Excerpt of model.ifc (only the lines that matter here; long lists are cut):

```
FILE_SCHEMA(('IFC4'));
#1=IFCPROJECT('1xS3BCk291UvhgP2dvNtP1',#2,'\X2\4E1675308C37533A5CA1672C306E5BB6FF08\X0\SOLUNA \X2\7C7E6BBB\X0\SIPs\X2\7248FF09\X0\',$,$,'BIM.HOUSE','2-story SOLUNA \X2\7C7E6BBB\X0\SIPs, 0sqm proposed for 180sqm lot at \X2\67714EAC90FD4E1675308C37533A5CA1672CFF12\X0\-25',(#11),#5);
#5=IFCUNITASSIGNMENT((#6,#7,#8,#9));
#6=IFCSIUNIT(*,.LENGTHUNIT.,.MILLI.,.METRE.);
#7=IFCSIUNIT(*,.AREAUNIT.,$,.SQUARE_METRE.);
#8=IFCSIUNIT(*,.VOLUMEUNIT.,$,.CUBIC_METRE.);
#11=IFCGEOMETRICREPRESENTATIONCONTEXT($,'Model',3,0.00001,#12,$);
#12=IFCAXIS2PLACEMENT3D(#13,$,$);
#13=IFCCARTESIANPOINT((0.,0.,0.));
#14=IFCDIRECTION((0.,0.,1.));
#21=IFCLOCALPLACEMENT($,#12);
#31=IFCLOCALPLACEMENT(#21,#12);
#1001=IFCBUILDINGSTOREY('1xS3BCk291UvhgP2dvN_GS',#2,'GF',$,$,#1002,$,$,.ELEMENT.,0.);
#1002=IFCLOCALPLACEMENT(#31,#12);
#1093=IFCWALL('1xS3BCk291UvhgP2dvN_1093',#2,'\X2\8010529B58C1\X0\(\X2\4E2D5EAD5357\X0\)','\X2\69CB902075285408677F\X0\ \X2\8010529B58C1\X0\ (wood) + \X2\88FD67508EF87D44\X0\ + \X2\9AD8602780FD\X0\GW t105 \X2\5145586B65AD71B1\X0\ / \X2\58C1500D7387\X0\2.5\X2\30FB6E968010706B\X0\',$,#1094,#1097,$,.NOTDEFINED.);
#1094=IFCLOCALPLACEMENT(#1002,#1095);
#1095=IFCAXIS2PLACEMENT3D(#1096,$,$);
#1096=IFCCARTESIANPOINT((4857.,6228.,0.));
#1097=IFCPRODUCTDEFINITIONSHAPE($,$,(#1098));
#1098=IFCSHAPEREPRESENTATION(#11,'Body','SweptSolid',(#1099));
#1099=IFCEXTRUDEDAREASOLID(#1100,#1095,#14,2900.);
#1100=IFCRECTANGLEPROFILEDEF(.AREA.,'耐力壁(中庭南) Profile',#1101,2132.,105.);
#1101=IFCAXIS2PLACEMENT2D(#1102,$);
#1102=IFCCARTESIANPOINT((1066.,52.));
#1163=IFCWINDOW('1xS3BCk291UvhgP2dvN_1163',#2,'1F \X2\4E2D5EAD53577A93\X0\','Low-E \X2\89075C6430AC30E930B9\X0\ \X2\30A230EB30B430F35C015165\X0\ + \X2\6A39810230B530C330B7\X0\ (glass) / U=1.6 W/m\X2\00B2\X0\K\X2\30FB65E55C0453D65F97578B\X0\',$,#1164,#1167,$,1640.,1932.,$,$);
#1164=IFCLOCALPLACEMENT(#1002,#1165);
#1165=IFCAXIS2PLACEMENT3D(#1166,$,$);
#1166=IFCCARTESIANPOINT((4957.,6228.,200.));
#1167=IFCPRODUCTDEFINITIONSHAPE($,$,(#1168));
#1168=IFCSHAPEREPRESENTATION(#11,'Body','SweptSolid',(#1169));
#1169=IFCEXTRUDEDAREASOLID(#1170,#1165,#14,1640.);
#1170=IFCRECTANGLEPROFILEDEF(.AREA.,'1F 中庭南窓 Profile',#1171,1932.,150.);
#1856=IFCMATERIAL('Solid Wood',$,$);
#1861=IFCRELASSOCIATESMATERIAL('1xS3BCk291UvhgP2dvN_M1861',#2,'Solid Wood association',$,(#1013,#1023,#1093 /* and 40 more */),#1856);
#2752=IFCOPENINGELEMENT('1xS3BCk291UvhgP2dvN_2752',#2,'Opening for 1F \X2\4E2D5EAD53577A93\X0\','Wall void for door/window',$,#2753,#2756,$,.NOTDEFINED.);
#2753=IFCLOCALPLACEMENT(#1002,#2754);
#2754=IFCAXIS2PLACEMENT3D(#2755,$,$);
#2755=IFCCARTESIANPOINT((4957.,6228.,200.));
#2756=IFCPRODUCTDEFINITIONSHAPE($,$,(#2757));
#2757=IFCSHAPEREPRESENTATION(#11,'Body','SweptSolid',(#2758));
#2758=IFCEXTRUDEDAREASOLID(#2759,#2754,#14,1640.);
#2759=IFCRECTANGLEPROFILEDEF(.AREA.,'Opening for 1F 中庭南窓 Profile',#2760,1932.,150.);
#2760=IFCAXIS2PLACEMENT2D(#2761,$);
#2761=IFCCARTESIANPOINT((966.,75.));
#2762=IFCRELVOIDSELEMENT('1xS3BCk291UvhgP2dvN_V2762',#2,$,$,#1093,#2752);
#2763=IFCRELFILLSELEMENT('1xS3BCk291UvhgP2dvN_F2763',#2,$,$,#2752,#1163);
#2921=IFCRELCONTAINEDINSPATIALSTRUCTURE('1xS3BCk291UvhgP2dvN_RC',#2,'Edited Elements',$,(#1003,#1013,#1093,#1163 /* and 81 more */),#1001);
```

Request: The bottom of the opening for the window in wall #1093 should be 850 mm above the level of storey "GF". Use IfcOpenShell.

```python
import numpy as np
import ifcopenshell
import ifcopenshell.api.geometry
import ifcopenshell.geom
import ifcopenshell.util.element
import ifcopenshell.util.placement
import ifcopenshell.util.shape
import ifcopenshell.util.unit

model = ifcopenshell.open("model.ifc")
unit_scale = ifcopenshell.util.unit.calculate_unit_scale(model)

window = model.by_guid("1xS3BCk291UvhgP2dvN_1163")
opening = window.FillsVoids[0].RelatingOpeningElement
storey = ifcopenshell.util.element.get_container(window, ifc_class="IfcBuildingStorey")
level = ifcopenshell.util.placement.get_local_placement(storey.ObjectPlacement)[2, 3]

# The opening's origin need not be at the sill, so measure its lowest point.
shape = ifcopenshell.geom.create_shape(ifcopenshell.geom.settings(), opening)
bottom = ifcopenshell.util.shape.get_shape_bottom_elevation(shape, shape.geometry) / unit_scale
dz = level + 0.85 / unit_scale - bottom

shift = np.array([0.0, 0.0, dz])
# The window is not placed relative to its opening, so move both.
for product in (opening, window):
    matrix = ifcopenshell.util.placement.get_local_placement(product.ObjectPlacement)
    matrix[:3, 3] += shift
    ifcopenshell.api.geometry.edit_object_placement(model, product=product, matrix=matrix, is_si=False)

print(f"moved by {dz * unit_scale:+.3f} m")

model.write("model_updated.ifc")
```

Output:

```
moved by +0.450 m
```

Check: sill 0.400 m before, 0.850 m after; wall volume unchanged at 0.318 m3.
